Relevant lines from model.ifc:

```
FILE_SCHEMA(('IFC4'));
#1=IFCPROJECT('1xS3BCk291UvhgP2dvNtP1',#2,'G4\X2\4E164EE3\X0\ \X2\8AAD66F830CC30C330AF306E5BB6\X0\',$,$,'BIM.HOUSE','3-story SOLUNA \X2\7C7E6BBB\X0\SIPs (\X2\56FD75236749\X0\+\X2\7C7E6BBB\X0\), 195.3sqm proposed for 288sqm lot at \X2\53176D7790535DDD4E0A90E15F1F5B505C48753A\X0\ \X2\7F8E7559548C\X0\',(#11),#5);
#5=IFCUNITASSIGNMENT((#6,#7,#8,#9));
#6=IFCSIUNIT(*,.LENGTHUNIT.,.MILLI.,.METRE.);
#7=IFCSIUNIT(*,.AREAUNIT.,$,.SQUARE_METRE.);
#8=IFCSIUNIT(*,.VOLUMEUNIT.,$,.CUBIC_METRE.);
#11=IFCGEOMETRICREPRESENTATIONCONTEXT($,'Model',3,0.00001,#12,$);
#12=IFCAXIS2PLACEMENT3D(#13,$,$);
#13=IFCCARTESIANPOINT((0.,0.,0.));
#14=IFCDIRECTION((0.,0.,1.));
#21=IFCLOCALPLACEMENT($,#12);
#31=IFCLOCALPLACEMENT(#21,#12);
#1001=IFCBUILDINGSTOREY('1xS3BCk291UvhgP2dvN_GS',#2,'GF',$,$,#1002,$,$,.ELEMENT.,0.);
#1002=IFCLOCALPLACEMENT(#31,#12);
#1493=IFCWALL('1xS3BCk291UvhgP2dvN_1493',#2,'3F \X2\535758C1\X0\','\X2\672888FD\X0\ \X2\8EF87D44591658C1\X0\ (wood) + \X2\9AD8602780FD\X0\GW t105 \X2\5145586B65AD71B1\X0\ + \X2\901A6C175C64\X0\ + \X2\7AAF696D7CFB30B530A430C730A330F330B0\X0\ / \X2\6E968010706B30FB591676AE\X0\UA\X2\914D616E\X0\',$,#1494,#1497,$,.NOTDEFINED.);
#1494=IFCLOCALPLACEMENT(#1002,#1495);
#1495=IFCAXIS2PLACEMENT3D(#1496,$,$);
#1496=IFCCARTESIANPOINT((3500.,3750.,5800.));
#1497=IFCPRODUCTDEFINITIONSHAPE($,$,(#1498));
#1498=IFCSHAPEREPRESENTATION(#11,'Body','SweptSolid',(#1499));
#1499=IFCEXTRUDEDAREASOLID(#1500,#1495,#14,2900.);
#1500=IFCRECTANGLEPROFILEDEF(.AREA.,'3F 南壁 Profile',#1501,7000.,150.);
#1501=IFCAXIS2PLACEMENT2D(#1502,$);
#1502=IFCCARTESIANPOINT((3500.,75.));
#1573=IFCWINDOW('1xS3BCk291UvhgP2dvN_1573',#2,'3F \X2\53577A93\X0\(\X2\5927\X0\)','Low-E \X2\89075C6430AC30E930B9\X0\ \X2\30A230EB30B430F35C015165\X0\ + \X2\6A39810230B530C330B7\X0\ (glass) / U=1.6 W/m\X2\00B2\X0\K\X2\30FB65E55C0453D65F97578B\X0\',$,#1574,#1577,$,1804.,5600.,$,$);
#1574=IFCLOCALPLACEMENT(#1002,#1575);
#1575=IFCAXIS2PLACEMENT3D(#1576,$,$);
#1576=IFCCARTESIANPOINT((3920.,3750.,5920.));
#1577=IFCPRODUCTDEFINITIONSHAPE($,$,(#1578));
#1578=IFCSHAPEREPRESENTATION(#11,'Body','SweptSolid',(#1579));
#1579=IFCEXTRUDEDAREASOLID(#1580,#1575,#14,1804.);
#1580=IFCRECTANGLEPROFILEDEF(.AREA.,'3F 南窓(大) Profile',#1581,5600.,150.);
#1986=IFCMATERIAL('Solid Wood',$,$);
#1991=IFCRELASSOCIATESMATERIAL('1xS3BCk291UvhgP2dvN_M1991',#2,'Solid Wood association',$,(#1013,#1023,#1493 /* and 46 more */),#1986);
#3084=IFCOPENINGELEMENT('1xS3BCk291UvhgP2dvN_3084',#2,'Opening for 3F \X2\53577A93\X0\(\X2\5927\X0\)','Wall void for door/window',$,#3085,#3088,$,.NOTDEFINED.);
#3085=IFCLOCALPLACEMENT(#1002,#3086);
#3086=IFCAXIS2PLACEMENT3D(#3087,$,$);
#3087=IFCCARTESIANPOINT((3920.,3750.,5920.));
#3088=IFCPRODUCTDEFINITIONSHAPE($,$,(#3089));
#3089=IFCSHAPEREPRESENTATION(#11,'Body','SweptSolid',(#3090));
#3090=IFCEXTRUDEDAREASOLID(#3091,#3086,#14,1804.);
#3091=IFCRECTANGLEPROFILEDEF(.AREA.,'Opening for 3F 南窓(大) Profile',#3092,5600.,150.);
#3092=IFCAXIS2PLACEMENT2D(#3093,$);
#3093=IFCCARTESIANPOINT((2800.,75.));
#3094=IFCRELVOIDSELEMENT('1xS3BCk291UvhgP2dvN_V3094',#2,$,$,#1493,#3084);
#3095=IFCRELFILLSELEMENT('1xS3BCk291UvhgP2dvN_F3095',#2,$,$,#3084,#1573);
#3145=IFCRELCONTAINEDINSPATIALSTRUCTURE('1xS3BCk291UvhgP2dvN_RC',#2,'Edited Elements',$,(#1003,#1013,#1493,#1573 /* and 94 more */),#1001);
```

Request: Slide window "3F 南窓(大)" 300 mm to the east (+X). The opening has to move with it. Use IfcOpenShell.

```python
import ifcopenshell
import ifcopenshell.api.geometry
import ifcopenshell.util.placement

model = ifcopenshell.open("model.ifc")

window = model.by_guid("1xS3BCk291UvhgP2dvN_1573")
opening = window.FillsVoids[0].RelatingOpeningElement
wall = opening.VoidsElements[0].RelatingBuildingElement

wall_matrix = ifcopenshell.util.placement.get_local_placement(wall.ObjectPlacement)
shift = wall_matrix[:3, 0] * 300.0
before = ifcopenshell.util.placement.get_local_placement(window.ObjectPlacement)[:3, 3].copy()

# The window is not placed relative to its opening, so move both.
for product in (opening, window):
    matrix = ifcopenshell.util.placement.get_local_placement(product.ObjectPlacement)
    matrix[:3, 3] += shift
    ifcopenshell.api.geometry.edit_object_placement(model, product=product, matrix=matrix, is_si=False)

after = ifcopenshell.util.placement.get_local_placement(window.ObjectPlacement)[:3, 3]
print("window moved by", (after - before).round(3) + 0.0)

model.write("model_v2.ifc")
```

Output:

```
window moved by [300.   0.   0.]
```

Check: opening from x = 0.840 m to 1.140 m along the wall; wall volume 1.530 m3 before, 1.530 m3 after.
